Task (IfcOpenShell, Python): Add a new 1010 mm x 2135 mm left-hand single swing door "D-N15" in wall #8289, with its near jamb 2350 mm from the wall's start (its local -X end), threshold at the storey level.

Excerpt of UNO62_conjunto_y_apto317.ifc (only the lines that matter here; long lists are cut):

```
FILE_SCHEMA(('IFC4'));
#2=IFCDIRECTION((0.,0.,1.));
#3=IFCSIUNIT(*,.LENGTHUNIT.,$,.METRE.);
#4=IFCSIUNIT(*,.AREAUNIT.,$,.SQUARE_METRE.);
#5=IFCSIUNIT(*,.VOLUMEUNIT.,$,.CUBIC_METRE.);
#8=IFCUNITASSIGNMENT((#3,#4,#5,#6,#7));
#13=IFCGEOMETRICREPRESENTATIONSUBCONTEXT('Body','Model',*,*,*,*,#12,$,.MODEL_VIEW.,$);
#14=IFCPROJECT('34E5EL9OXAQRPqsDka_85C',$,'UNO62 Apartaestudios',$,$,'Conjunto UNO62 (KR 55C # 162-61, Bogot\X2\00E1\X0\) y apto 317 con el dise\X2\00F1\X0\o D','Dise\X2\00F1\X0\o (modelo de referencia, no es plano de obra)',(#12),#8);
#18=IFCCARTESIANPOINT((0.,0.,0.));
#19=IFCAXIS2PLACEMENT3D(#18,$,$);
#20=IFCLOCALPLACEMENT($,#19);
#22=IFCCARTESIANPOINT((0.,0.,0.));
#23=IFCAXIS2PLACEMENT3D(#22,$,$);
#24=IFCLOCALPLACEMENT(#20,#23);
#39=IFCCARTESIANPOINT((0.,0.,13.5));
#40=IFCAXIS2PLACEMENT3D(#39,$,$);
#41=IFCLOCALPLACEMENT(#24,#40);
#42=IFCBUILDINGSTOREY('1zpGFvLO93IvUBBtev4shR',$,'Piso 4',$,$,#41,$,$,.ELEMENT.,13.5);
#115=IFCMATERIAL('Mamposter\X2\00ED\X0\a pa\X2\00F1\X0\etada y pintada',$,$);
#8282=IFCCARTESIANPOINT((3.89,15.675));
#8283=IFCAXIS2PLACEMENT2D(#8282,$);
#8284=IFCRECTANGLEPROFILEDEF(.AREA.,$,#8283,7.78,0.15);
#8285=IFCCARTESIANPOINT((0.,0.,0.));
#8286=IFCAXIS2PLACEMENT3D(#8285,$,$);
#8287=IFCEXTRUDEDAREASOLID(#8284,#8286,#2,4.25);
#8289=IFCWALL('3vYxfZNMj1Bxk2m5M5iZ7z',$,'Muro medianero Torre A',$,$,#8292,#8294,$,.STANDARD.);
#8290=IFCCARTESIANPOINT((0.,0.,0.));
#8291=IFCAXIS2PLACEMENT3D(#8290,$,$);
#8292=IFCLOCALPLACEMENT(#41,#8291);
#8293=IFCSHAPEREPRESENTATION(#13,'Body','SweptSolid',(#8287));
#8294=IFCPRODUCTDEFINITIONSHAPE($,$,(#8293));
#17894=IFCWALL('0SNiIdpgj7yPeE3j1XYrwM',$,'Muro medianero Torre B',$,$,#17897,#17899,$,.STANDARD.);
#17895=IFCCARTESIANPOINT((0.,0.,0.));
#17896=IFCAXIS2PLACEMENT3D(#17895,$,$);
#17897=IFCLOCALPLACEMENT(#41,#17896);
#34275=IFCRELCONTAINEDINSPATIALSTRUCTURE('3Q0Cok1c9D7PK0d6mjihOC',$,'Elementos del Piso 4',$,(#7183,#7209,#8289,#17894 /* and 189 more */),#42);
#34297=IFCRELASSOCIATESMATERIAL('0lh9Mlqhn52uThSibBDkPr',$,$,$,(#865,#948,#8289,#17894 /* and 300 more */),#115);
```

```python
import numpy as np
import ifcopenshell
import ifcopenshell.api.feature
import ifcopenshell.api.geometry
import ifcopenshell.api.root
import ifcopenshell.api.spatial
import ifcopenshell.geom
import ifcopenshell.util.element
import ifcopenshell.util.placement
import ifcopenshell.util.representation
import ifcopenshell.util.shape
import ifcopenshell.util.unit

model = ifcopenshell.open("UNO62_conjunto_y_apto317.ifc")
unit_scale = ifcopenshell.util.unit.calculate_unit_scale(model)
settings = ifcopenshell.geom.settings()


def volume(element):
    """Net volume in cubic metres, openings subtracted."""
    shape = ifcopenshell.geom.create_shape(settings, element)
    return ifcopenshell.util.shape.get_volume(shape.geometry)


wall = model.by_id(8289)
storey = ifcopenshell.util.element.get_container(wall, ifc_class="IfcBuildingStorey")
context = ifcopenshell.util.representation.get_context(model, "Model", "Body", "MODEL_VIEW")
before = volume(wall)

width, height, from_end, sill = 1.01, 2.135, 2.35, 0.0  # metres

# The wall runs along its own X axis, and the end named is its -X end.
wall_shape = ifcopenshell.geom.create_shape(settings, wall)
x, y, z = ifcopenshell.util.shape.get_vertices(wall_shape.geometry).T
start = x.min() + from_end
face, thickness = float(y.min()), float(y.max() - y.min())
wall_matrix = ifcopenshell.util.placement.get_local_placement(wall.ObjectPlacement)
level = ifcopenshell.util.placement.get_local_placement(storey.ObjectPlacement)[2, 3]


def in_wall(x, y):
    """Placement at x, y metres in the wall's axes, at sill height."""
    matrix = wall_matrix.copy()
    matrix[:, 3] = wall_matrix @ np.array([x / unit_scale, y / unit_scale, 0.0, 1.0])
    matrix[2, 3] = level + sill / unit_scale
    return matrix


# Opening: a box that overshoots both wall faces by 50 mm.
opening = ifcopenshell.api.root.create_entity(model, ifc_class="IfcOpeningElement", predefined_type="OPENING")
box = ifcopenshell.api.geometry.add_wall_representation(
    model, context=context, length=width, height=height, thickness=thickness + 0.1
)
ifcopenshell.api.geometry.assign_representation(model, product=opening, representation=box)
ifcopenshell.api.geometry.edit_object_placement(model, product=opening, matrix=in_wall(start, face - 0.05), is_si=False)
ifcopenshell.api.feature.add_feature(model, feature=opening, element=wall)

door = ifcopenshell.api.root.create_entity(model, ifc_class="IfcDoor", name="D-N15", predefined_type="DOOR")
door.OverallWidth, door.OverallHeight = width / unit_scale, height / unit_scale
door.OperationType = "SINGLE_SWING_LEFT"
body = ifcopenshell.api.geometry.add_door_representation(
    model,
    context=context,
    overall_width=door.OverallWidth,
    overall_height=door.OverallHeight,
    operation_type="SINGLE_SWING_LEFT",
    lining_properties={"LiningDepth": thickness / unit_scale, "ThresholdDepth": thickness / unit_scale},
)
ifcopenshell.api.geometry.assign_representation(model, product=door, representation=body)
ifcopenshell.api.spatial.assign_container(model, products=[door], relating_structure=storey)
ifcopenshell.api.feature.add_filling(model, opening=opening, element=door)

# The lining spans the wall, so the door starts at the wall face.
ifcopenshell.api.geometry.edit_object_placement(model, product=door, matrix=in_wall(start, face), is_si=False)

after = volume(wall)

print(f"wall volume {before:.3f} -> {after:.3f} m3")

model.write("UNO62_conjunto_y_apto317-out.ifc")
```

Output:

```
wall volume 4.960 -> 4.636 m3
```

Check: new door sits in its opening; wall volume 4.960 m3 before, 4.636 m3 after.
